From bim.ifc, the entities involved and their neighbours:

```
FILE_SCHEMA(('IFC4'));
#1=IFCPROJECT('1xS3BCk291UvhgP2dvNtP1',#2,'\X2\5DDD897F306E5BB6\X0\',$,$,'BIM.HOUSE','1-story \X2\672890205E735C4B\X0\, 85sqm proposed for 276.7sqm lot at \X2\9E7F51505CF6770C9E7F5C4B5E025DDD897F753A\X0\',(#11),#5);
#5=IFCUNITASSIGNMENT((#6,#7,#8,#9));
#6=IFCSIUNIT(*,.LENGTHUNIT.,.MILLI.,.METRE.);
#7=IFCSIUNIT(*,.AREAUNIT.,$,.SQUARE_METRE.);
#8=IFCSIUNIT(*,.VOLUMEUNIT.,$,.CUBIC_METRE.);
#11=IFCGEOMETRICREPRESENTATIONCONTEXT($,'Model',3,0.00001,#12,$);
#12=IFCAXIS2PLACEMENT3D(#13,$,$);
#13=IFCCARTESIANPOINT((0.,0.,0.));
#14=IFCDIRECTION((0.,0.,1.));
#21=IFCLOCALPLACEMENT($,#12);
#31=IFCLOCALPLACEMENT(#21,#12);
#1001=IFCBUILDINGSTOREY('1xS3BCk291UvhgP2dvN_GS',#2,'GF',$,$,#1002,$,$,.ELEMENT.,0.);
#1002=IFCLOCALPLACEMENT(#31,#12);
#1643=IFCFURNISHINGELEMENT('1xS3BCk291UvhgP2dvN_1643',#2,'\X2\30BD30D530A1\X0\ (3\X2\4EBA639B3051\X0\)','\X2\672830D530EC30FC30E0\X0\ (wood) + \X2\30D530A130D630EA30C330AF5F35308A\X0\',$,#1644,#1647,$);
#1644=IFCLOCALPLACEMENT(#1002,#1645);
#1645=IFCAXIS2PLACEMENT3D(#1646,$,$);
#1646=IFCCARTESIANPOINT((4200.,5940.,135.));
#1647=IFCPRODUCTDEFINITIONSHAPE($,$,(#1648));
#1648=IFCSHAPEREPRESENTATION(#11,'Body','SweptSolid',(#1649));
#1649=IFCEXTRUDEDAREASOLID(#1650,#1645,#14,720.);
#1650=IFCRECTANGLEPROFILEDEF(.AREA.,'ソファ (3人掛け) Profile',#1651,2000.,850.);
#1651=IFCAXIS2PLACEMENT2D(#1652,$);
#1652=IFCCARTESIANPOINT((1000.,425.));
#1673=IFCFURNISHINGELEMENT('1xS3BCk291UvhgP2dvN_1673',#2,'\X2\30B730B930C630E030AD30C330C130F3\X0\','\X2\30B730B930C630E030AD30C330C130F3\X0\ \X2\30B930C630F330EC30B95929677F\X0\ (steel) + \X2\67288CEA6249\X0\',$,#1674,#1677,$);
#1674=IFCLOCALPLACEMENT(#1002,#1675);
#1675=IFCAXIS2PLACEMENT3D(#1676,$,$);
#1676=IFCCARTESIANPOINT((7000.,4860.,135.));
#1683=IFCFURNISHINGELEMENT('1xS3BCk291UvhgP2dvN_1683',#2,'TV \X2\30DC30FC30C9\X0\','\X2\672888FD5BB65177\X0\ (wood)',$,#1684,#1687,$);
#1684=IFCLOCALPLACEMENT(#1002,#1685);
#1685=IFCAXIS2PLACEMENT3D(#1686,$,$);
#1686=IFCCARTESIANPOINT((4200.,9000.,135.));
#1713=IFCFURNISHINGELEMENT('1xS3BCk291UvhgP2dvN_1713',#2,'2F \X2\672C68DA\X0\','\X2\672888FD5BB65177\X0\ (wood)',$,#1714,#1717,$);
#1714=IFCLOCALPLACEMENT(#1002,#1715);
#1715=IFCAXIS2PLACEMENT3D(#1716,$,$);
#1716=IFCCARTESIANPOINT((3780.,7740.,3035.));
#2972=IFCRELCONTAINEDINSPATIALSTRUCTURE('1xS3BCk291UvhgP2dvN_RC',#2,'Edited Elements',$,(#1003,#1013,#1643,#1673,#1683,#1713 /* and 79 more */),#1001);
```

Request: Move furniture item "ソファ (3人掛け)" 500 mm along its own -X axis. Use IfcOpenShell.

```python
import ifcopenshell
import ifcopenshell.api.geometry
import ifcopenshell.util.placement
import ifcopenshell.util.unit

model = ifcopenshell.open("bim.ifc")
unit_scale = ifcopenshell.util.unit.calculate_unit_scale(model)

item = model.by_guid("1xS3BCk291UvhgP2dvN_1643")
matrix = ifcopenshell.util.placement.get_local_placement(item.ObjectPlacement)
matrix[:3, 3] -= matrix[:3, 0] * 0.5 / unit_scale
ifcopenshell.api.geometry.edit_object_placement(model, product=item, matrix=matrix, is_si=False)

print(ifcopenshell.util.placement.get_local_placement(item.ObjectPlacement).round(3) + 0.0)

model.write("bim_v2.ifc")
```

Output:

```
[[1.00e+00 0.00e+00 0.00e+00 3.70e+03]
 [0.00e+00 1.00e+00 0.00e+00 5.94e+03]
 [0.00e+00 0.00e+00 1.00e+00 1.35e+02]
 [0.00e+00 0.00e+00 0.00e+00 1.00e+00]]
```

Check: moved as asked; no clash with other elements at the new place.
